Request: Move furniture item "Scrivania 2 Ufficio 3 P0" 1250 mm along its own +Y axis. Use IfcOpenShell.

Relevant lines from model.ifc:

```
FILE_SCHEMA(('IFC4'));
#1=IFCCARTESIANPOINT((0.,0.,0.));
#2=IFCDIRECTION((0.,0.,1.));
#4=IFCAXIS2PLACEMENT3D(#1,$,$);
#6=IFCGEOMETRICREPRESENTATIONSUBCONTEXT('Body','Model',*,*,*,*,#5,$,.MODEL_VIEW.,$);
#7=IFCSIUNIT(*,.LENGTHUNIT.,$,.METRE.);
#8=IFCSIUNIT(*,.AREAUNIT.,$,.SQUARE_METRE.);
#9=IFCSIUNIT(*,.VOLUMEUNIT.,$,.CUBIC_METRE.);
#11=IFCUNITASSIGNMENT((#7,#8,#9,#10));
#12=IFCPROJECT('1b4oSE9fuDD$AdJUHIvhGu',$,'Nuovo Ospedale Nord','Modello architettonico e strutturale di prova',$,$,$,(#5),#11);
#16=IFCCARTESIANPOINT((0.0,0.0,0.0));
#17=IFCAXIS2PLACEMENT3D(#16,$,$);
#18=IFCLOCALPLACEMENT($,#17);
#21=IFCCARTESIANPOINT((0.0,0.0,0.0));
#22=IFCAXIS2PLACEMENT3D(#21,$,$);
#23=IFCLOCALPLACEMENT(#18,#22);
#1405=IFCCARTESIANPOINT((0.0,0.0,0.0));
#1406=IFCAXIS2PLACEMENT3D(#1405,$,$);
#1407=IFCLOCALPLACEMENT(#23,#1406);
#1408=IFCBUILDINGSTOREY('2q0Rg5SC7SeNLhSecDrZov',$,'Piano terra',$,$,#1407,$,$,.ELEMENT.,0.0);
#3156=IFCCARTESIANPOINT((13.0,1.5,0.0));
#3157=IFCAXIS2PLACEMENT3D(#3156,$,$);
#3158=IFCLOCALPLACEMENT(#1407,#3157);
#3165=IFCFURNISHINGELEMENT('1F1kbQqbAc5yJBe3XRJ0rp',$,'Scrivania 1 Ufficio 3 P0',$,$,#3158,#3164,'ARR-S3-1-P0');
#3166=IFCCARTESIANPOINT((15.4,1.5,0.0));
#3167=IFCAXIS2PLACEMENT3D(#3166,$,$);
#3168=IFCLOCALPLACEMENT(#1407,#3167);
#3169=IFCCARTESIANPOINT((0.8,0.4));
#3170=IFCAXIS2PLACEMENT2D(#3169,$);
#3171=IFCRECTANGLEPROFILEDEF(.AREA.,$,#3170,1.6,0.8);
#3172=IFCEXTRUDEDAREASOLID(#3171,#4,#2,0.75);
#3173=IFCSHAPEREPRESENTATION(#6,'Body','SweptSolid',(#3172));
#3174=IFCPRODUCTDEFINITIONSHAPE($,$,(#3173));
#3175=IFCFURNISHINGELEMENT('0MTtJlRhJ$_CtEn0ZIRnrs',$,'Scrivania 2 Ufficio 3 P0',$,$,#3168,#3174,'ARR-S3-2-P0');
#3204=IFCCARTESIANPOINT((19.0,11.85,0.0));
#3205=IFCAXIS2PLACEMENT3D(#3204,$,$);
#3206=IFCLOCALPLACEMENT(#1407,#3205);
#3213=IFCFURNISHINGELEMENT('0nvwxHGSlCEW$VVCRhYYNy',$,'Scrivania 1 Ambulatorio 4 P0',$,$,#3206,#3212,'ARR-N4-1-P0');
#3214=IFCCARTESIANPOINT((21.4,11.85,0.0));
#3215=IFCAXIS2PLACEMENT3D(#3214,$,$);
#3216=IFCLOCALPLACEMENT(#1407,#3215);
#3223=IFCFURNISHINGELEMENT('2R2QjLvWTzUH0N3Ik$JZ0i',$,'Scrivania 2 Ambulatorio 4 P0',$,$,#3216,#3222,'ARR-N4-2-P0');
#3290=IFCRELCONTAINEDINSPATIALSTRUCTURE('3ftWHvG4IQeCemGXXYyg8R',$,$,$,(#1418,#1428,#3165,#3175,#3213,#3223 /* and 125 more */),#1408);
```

```python
import ifcopenshell
import ifcopenshell.api.geometry
import ifcopenshell.util.placement
import ifcopenshell.util.unit

model = ifcopenshell.open("model.ifc")
unit_scale = ifcopenshell.util.unit.calculate_unit_scale(model)

item = model.by_guid("0MTtJlRhJ$_CtEn0ZIRnrs")
matrix = ifcopenshell.util.placement.get_local_placement(item.ObjectPlacement)
matrix[:3, 3] += matrix[:3, 1] * 1.25 / unit_scale
ifcopenshell.api.geometry.edit_object_placement(model, product=item, matrix=matrix, is_si=False)

print(ifcopenshell.util.placement.get_local_placement(item.ObjectPlacement).round(3) + 0.0)

model.write("model-out.ifc")
```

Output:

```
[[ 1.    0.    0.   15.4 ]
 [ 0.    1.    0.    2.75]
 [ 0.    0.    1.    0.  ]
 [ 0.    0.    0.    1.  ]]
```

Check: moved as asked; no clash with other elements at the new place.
